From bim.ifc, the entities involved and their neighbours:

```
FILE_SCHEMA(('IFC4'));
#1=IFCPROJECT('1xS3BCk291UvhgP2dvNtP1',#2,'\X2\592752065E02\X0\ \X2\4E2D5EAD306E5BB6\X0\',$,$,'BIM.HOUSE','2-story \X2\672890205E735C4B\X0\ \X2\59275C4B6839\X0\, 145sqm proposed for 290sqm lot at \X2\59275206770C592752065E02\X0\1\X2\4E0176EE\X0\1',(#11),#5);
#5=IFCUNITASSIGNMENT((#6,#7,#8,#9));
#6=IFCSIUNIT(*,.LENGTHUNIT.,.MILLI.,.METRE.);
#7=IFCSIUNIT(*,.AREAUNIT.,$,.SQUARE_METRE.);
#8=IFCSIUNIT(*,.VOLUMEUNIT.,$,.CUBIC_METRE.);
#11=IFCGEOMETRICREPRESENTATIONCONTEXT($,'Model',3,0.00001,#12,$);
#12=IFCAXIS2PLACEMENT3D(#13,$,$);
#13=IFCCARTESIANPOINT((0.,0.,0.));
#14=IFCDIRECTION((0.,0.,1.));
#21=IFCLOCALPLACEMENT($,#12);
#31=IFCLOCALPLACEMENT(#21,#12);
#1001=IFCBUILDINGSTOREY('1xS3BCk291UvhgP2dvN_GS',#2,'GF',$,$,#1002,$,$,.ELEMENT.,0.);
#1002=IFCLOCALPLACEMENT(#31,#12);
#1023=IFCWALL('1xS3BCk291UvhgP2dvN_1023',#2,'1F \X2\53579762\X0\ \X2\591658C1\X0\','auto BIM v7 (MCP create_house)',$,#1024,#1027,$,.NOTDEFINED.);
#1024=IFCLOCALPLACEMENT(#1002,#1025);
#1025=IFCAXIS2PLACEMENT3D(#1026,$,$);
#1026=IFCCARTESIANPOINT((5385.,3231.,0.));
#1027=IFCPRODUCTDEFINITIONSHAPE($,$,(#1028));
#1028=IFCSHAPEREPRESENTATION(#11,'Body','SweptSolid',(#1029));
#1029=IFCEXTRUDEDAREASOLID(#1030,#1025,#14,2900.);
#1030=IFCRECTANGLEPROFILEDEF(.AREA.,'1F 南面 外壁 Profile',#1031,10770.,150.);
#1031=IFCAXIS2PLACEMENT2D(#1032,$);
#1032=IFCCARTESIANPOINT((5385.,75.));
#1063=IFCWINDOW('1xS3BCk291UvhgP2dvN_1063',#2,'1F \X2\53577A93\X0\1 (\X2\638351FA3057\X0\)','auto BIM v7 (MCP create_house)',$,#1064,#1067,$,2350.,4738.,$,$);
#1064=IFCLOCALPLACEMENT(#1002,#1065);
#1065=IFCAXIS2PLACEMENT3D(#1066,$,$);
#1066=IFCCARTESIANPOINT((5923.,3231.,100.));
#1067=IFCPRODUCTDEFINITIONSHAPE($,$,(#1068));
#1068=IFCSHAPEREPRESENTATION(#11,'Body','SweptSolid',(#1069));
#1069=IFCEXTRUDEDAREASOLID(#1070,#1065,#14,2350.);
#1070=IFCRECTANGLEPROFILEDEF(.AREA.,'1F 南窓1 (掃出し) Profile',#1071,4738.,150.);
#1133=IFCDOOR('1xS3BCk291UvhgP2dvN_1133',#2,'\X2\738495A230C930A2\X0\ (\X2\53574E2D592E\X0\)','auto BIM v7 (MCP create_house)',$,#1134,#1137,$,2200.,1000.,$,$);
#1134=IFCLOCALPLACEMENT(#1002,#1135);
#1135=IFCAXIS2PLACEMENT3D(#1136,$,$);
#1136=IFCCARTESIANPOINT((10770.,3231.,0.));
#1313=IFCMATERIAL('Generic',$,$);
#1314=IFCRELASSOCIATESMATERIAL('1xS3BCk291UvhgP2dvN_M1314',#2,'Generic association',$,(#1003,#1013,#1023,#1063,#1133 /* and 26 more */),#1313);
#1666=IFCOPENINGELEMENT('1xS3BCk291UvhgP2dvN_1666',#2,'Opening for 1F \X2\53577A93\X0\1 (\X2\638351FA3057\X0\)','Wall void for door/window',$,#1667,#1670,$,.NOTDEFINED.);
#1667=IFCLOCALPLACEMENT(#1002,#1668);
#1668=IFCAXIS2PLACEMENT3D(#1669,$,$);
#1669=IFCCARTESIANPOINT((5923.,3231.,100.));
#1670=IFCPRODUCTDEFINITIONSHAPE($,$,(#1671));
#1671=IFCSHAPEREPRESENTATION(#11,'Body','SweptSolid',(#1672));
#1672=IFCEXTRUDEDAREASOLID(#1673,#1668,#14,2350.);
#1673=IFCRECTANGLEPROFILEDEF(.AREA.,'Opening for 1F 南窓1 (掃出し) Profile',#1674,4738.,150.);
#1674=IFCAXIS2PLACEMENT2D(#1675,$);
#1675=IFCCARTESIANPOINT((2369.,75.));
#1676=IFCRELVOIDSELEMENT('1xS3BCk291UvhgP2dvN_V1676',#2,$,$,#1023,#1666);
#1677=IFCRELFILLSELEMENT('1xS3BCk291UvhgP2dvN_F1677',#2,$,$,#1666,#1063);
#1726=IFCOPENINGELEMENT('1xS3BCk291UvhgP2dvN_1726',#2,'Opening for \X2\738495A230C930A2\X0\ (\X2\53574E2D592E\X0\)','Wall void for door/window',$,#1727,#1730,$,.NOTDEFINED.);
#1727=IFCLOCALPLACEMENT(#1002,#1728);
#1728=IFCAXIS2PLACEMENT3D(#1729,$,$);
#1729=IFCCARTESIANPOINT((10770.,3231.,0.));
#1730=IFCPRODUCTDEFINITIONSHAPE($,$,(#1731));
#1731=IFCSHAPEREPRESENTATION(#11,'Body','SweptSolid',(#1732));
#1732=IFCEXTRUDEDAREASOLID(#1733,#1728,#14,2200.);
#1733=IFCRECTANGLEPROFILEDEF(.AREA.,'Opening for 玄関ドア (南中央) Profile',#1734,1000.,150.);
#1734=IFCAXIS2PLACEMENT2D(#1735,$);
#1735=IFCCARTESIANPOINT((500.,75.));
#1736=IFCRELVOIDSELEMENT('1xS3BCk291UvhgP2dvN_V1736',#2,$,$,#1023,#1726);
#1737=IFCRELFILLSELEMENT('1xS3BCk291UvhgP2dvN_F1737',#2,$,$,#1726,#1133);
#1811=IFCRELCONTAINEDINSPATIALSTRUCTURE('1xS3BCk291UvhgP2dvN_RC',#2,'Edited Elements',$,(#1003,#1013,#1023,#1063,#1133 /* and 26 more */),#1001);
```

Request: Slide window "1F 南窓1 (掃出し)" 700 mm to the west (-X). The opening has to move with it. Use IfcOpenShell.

```python
import ifcopenshell
import ifcopenshell.api.geometry
import ifcopenshell.util.placement
import ifcopenshell.util.unit

model = ifcopenshell.open("bim.ifc")
unit_scale = ifcopenshell.util.unit.calculate_unit_scale(model)

window = model.by_guid("1xS3BCk291UvhgP2dvN_1063")
opening = window.FillsVoids[0].RelatingOpeningElement
wall = opening.VoidsElements[0].RelatingBuildingElement

wall_matrix = ifcopenshell.util.placement.get_local_placement(wall.ObjectPlacement)
shift = wall_matrix[:3, 0] * -0.7 / unit_scale
before = ifcopenshell.util.placement.get_local_placement(window.ObjectPlacement)[:3, 3].copy()

# The window is not placed relative to its opening, so move both.
for product in (opening, window):
    matrix = ifcopenshell.util.placement.get_local_placement(product.ObjectPlacement)
    matrix[:3, 3] += shift
    ifcopenshell.api.geometry.edit_object_placement(model, product=product, matrix=matrix, is_si=False)

after = ifcopenshell.util.placement.get_local_placement(window.ObjectPlacement)[:3, 3]
print("window moved by", (after - before).round(3) + 0.0)

model.write("bim_edited.ifc")
```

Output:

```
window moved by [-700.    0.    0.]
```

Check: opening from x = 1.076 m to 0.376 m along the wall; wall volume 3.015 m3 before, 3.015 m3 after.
